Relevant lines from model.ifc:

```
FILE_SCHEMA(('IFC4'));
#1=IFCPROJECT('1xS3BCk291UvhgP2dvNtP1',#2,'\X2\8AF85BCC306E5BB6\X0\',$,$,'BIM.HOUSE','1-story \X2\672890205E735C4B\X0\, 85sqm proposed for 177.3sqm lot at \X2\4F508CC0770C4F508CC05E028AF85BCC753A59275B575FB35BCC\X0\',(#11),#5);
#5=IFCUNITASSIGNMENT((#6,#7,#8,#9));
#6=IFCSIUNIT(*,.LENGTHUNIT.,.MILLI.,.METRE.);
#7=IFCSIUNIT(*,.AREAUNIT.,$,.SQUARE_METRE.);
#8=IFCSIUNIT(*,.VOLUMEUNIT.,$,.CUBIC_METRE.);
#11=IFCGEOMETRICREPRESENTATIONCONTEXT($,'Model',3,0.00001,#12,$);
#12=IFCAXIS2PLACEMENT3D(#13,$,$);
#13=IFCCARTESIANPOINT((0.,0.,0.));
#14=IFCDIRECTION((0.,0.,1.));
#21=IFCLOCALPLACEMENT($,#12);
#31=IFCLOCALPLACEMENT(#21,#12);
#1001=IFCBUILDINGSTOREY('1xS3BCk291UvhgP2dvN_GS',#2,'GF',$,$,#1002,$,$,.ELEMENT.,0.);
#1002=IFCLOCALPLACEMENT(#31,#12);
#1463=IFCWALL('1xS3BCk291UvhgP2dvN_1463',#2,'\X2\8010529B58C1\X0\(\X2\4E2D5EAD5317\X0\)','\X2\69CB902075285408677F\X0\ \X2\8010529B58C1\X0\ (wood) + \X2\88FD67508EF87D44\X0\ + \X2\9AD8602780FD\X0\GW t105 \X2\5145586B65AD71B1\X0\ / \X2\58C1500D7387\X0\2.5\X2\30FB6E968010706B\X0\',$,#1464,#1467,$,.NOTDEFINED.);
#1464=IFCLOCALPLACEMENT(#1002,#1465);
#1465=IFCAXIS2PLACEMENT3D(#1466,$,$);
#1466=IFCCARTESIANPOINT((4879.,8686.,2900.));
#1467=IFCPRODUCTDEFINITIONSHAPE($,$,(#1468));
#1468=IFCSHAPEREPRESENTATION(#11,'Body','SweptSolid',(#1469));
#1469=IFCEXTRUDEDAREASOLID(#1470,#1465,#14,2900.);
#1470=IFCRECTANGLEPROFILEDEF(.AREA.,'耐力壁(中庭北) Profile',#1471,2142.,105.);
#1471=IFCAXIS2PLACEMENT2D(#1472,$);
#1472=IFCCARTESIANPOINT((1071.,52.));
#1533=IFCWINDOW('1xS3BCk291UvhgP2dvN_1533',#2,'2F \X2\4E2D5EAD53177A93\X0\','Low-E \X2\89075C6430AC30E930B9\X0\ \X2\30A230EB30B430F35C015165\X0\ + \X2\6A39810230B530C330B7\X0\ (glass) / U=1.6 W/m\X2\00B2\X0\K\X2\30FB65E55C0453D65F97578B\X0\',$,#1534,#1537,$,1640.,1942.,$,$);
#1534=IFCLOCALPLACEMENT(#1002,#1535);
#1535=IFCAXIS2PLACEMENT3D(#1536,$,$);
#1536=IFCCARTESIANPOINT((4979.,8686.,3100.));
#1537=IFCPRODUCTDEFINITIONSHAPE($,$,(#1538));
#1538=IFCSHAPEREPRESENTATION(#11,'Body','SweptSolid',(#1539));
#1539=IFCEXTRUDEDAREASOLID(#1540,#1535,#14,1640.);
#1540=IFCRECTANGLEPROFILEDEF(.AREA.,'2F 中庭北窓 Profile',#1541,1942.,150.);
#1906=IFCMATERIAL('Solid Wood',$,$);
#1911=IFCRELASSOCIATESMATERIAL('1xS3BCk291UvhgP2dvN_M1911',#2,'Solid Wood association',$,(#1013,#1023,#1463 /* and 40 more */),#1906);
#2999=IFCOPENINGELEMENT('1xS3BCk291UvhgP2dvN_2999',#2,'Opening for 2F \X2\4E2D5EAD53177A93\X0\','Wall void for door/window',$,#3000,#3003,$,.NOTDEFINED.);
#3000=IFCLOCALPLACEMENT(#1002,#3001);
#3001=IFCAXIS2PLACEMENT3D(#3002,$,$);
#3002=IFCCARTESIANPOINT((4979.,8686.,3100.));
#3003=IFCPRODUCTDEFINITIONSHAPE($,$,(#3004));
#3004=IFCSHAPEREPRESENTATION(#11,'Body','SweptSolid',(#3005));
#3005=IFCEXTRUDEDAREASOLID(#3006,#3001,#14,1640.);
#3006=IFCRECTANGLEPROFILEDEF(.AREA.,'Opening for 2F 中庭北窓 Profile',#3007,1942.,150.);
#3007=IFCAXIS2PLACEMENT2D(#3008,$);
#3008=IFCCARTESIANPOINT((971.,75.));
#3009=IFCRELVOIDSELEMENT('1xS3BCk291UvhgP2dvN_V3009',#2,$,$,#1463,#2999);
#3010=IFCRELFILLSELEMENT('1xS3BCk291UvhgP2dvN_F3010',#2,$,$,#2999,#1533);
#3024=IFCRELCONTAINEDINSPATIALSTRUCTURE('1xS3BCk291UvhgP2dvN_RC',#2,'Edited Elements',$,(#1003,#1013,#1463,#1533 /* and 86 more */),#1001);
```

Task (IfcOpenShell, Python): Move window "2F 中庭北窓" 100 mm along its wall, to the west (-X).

```python
import ifcopenshell
import ifcopenshell.api.geometry
import ifcopenshell.util.placement

model = ifcopenshell.open("model.ifc")

window = model.by_guid("1xS3BCk291UvhgP2dvN_1533")
opening = window.FillsVoids[0].RelatingOpeningElement
wall = opening.VoidsElements[0].RelatingBuildingElement

wall_matrix = ifcopenshell.util.placement.get_local_placement(wall.ObjectPlacement)
shift = wall_matrix[:3, 0] * -100.0
before = ifcopenshell.util.placement.get_local_placement(window.ObjectPlacement)[:3, 3].copy()

# The window is not placed relative to its opening, so move both.
for product in (opening, window):
    matrix = ifcopenshell.util.placement.get_local_placement(product.ObjectPlacement)
    matrix[:3, 3] += shift
    ifcopenshell.api.geometry.edit_object_placement(model, product=product, matrix=matrix, is_si=False)

after = ifcopenshell.util.placement.get_local_placement(window.ObjectPlacement)[:3, 3]
print("window moved by", (after - before).round(3) + 0.0)

model.write("model_updated.ifc")
```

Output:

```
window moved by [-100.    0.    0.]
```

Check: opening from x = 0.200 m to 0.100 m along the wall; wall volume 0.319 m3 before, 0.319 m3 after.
